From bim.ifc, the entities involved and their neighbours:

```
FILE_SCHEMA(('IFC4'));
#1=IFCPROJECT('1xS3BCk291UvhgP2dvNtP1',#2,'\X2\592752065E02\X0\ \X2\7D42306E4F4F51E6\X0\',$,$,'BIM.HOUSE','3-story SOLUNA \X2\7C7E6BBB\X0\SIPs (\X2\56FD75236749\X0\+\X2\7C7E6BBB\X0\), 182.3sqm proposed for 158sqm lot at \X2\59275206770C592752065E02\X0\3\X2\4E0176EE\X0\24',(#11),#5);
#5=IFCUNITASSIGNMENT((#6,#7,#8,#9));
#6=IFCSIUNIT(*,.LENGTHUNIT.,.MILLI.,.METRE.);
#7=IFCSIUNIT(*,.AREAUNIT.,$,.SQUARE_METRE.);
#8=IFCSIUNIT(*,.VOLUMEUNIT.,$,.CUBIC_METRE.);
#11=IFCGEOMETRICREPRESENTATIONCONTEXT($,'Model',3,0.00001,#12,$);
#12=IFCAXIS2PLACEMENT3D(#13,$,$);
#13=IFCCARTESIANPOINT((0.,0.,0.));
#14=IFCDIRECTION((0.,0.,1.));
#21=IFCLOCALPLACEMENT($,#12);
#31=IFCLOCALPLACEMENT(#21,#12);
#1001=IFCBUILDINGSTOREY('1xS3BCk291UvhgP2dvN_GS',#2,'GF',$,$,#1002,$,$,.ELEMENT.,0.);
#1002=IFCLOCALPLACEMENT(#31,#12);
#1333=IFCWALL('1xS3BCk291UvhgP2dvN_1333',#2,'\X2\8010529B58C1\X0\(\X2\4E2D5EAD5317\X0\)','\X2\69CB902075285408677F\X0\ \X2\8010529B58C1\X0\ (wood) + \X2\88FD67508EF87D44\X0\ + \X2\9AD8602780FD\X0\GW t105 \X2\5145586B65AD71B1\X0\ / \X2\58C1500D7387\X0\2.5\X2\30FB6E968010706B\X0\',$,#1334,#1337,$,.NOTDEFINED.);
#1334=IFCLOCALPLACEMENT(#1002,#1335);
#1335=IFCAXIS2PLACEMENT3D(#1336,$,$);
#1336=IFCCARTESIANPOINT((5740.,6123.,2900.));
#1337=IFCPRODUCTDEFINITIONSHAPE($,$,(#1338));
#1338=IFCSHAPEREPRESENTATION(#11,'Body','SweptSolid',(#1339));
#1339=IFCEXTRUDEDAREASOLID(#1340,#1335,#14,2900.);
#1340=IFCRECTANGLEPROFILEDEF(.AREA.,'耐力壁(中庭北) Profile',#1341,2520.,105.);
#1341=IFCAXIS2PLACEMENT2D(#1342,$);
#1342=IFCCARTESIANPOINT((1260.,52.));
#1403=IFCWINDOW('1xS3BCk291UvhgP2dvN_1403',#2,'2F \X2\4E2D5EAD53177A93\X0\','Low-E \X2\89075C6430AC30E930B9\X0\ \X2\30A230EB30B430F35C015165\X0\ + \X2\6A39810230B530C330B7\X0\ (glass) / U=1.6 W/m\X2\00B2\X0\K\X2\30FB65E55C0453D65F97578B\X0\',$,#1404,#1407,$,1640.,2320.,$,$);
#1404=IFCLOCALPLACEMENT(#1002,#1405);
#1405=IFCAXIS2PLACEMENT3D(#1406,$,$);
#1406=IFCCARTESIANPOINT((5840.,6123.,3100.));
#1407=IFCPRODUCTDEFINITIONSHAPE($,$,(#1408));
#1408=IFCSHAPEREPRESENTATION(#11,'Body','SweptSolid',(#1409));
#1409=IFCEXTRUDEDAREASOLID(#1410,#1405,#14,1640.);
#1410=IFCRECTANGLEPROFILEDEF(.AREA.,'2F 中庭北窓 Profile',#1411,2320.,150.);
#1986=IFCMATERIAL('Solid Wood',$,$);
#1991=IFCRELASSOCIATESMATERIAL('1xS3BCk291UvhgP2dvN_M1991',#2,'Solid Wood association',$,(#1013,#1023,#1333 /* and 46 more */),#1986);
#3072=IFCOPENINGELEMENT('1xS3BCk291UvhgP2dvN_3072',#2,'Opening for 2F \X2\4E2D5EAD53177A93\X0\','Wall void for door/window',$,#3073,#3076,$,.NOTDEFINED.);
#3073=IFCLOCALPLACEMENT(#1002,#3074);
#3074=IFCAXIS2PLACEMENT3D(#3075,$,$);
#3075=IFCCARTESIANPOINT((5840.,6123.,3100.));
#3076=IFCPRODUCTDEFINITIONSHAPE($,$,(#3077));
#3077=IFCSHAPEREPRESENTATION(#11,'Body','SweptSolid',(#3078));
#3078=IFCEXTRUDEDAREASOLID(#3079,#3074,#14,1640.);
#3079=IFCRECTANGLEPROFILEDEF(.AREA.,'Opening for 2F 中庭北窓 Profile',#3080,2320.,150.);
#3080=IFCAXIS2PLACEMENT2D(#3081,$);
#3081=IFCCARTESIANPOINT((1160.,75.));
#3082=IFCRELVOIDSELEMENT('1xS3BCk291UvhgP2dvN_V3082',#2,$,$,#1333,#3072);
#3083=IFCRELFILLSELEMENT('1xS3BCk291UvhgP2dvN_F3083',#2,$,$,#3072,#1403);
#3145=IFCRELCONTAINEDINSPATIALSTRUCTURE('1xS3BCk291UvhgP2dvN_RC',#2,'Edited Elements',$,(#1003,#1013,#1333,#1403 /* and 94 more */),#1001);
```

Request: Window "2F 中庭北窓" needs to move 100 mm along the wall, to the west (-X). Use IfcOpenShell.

```python
import ifcopenshell
import ifcopenshell.api.geometry
import ifcopenshell.util.placement

model = ifcopenshell.open("bim.ifc")

window = model.by_guid("1xS3BCk291UvhgP2dvN_1403")
opening = window.FillsVoids[0].RelatingOpeningElement
wall = opening.VoidsElements[0].RelatingBuildingElement

wall_matrix = ifcopenshell.util.placement.get_local_placement(wall.ObjectPlacement)
shift = wall_matrix[:3, 0] * -100.0
before = ifcopenshell.util.placement.get_local_placement(window.ObjectPlacement)[:3, 3].copy()

# The window is not placed relative to its opening, so move both.
for product in (opening, window):
    matrix = ifcopenshell.util.placement.get_local_placement(product.ObjectPlacement)
    matrix[:3, 3] += shift
    ifcopenshell.api.geometry.edit_object_placement(model, product=product, matrix=matrix, is_si=False)

after = ifcopenshell.util.placement.get_local_placement(window.ObjectPlacement)[:3, 3]
print("window moved by", (after - before).round(3) + 0.0)

model.write("bim_v2.ifc")
```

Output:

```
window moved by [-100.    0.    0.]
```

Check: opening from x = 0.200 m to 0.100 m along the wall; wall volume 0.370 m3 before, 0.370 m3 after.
